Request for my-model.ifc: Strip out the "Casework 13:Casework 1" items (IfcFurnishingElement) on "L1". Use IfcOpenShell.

First a look at what the model holds.

```python
import ifcopenshell
import ifcopenshell.util.element

model = ifcopenshell.open("my-model.ifc")
print(model.schema)
storey = next(s for s in model.by_type("IfcBuildingStorey") if s.Name == "L1")
furniture = [e for e in ifcopenshell.util.element.get_decomposition(storey) if e.is_a("IfcFurnishingElement")]
seen = {}
for e in furniture:
    element_type = ifcopenshell.util.element.get_type(e)
    name = element_type.Name if element_type not in (None, e) else None
    seen[name] = seen.get(name, 0) + 1
for name, count in sorted(seen.items(), key=str):
    print(count, "x", name)
```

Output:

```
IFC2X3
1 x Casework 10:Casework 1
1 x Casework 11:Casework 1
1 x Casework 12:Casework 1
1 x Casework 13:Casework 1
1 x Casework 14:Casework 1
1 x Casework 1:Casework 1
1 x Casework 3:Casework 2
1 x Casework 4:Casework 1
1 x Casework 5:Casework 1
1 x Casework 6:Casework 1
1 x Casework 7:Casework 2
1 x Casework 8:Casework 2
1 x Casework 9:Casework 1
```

```python
import ifcopenshell
import ifcopenshell.api.root
import ifcopenshell.util.element

model = ifcopenshell.open("my-model.ifc")

storey = next(s for s in model.by_type("IfcBuildingStorey") if s.Name == "L1")
furniture = [e for e in ifcopenshell.util.element.get_decomposition(storey) if e.is_a("IfcFurnishingElement")]
targets = [e for e in furniture if (t := ifcopenshell.util.element.get_type(e)) not in (None, e) and t.Name == "Casework 13:Casework 1"]

for e in targets:
    ifcopenshell.api.root.remove_product(model, product=e)
print(len(targets), "removed")

model.write("my-model_v2.ifc")
```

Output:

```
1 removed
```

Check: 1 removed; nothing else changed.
